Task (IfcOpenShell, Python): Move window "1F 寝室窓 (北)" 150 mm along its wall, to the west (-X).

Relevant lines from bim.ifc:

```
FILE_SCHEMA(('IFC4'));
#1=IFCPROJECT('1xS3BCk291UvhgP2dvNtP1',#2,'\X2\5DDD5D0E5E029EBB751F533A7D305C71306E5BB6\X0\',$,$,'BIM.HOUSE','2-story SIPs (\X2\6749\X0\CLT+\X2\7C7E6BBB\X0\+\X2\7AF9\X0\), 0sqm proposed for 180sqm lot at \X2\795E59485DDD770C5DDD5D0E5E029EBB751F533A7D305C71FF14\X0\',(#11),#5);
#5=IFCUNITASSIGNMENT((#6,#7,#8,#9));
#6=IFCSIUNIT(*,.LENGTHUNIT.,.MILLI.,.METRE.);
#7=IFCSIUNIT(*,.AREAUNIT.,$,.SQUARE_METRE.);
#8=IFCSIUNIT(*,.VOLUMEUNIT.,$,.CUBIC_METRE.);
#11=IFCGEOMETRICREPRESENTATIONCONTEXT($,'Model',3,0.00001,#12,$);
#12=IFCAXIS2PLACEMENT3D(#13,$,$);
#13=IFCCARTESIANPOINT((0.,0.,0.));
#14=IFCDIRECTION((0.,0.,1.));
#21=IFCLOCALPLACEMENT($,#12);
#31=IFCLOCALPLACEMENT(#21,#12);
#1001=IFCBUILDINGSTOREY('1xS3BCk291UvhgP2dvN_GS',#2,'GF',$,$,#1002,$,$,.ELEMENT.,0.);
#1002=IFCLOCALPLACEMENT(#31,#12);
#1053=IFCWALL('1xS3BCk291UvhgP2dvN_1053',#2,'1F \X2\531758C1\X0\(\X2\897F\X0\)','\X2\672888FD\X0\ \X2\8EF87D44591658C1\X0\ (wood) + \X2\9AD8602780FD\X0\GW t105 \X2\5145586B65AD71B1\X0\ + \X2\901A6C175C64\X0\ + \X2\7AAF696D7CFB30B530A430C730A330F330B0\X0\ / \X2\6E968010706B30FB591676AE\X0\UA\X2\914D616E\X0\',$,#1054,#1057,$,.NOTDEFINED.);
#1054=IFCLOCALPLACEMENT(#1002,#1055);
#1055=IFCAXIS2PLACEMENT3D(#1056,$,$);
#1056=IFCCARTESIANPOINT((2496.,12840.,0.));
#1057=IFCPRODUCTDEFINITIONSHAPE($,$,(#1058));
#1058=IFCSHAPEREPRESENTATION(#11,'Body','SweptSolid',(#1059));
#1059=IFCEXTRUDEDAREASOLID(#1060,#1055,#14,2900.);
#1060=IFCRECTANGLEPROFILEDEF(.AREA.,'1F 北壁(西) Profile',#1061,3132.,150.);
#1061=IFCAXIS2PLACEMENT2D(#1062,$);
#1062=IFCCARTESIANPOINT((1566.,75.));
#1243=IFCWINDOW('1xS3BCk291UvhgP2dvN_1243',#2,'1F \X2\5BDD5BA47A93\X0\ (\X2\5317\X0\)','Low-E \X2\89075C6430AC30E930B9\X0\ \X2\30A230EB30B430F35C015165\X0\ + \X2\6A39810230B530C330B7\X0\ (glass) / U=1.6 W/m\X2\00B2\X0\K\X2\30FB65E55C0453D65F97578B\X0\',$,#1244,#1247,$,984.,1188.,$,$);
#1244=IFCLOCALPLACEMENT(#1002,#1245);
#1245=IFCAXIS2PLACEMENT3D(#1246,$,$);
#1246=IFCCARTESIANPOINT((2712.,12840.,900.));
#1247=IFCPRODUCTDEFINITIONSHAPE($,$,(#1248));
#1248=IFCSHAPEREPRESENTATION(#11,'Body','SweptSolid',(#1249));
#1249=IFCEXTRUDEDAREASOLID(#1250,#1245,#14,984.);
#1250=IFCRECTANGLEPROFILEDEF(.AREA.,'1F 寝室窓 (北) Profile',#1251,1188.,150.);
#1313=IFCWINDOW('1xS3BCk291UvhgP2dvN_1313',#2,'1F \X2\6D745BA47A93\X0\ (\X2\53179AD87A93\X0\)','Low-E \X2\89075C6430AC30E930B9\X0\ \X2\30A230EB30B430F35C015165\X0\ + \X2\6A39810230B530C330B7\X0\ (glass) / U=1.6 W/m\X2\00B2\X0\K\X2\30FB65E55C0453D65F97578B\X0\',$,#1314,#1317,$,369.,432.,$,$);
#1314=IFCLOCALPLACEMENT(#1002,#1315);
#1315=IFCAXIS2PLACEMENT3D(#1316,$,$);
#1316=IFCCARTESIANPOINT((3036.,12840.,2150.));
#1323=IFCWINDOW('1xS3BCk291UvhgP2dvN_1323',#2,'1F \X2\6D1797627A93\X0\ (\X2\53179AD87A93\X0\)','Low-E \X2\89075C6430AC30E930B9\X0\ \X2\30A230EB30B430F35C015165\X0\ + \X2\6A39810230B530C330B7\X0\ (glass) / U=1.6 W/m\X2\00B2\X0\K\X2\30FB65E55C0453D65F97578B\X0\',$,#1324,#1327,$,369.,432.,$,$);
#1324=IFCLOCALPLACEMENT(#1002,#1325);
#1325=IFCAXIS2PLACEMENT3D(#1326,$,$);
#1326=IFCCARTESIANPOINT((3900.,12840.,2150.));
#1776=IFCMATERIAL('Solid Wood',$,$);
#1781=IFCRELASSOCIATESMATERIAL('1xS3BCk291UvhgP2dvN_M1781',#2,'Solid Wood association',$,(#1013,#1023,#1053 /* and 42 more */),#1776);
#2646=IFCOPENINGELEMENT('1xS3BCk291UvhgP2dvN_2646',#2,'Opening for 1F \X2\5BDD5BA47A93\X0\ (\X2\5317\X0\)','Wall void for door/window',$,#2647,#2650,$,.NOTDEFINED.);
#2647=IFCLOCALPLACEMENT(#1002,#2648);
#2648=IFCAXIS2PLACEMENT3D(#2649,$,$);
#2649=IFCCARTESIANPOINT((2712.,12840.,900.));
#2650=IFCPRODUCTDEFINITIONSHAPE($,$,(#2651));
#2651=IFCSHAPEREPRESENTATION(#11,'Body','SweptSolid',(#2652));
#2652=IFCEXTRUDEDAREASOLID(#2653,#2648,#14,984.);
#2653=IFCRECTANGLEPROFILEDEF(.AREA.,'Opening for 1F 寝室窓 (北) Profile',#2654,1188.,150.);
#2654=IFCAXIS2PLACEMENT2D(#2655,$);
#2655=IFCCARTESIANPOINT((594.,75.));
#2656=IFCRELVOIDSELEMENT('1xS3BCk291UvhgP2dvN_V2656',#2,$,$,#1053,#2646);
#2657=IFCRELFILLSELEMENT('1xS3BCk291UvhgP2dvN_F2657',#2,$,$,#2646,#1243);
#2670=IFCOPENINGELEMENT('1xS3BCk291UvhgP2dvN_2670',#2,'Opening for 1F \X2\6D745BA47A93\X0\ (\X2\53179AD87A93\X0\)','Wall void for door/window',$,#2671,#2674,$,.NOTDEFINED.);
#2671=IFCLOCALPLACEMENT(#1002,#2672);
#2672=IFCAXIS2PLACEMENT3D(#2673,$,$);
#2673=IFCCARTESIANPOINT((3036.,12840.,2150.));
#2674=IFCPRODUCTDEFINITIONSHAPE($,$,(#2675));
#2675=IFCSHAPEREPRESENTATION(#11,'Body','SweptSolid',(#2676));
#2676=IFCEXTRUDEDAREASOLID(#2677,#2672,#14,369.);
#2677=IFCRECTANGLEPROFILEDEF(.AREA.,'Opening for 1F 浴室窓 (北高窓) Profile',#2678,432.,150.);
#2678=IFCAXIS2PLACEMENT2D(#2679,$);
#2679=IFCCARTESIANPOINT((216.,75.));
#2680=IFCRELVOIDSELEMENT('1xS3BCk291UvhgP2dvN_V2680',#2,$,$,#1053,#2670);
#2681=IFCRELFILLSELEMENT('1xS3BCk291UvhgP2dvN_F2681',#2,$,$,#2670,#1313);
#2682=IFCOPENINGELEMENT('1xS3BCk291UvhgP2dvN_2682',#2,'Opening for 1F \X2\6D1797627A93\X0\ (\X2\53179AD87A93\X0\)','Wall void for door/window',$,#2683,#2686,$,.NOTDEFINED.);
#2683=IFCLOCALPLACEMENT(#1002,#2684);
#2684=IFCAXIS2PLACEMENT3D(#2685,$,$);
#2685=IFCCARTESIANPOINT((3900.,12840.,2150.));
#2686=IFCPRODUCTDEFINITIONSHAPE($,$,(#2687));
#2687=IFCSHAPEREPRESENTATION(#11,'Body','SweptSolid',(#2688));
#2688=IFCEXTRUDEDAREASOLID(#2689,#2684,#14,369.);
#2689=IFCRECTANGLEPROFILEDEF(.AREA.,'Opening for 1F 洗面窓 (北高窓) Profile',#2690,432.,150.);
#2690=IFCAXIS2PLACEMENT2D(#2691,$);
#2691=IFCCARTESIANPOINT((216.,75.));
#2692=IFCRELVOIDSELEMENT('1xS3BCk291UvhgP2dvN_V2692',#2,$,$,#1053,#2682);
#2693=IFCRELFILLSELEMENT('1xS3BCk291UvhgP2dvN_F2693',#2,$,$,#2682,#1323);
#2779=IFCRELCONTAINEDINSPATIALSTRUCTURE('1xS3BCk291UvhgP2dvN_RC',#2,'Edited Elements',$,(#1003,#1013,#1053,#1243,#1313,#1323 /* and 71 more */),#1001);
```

```python
import ifcopenshell
import ifcopenshell.api.geometry
import ifcopenshell.util.placement

model = ifcopenshell.open("bim.ifc")

window = model.by_id(1243)
opening = window.FillsVoids[0].RelatingOpeningElement
wall = opening.VoidsElements[0].RelatingBuildingElement

wall_matrix = ifcopenshell.util.placement.get_local_placement(wall.ObjectPlacement)
shift = wall_matrix[:3, 0] * -150.0
before = ifcopenshell.util.placement.get_local_placement(window.ObjectPlacement)[:3, 3].copy()

# The window is not placed relative to its opening, so move both.
for product in (opening, window):
    matrix = ifcopenshell.util.placement.get_local_placement(product.ObjectPlacement)
    matrix[:3, 3] += shift
    ifcopenshell.api.geometry.edit_object_placement(model, product=product, matrix=matrix, is_si=False)

after = ifcopenshell.util.placement.get_local_placement(window.ObjectPlacement)[:3, 3]
print("window moved by", (after - before).round(3) + 0.0)

model.write("bim_v2.ifc")
```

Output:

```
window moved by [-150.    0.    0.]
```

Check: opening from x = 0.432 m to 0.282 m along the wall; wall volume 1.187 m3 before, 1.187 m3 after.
